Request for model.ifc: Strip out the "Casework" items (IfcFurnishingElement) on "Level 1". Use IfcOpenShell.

First a look at what the model holds.

```python
import ifcopenshell
import ifcopenshell.util.element

model = ifcopenshell.open("model.ifc")
print(model.schema)
storey = next(s for s in model.by_type("IfcBuildingStorey") if s.Name == "Level 1")
furniture = [e for e in ifcopenshell.util.element.get_decomposition(storey) if e.is_a("IfcFurnishingElement")]
seen = {}
for e in furniture:
    element_type = ifcopenshell.util.element.get_type(e)
    name = element_type.Name if element_type not in (None, e) else None
    seen[name] = seen.get(name, 0) + 1
for name, count in sorted(seen.items(), key=str):
    print(count, "x", name)
```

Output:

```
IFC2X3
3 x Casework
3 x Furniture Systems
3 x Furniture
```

```python
import ifcopenshell
import ifcopenshell.api.root
import ifcopenshell.util.element

model = ifcopenshell.open("model.ifc")

storey = next(s for s in model.by_type("IfcBuildingStorey") if s.Name == "Level 1")
furniture = [e for e in ifcopenshell.util.element.get_decomposition(storey) if e.is_a("IfcFurnishingElement")]
targets = [e for e in furniture if (t := ifcopenshell.util.element.get_type(e)) not in (None, e) and t.Name == "Casework"]

for e in targets:
    ifcopenshell.api.root.remove_product(model, product=e)
print(len(targets), "removed")

model.write("model_v2.ifc")
```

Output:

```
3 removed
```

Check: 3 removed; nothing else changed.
